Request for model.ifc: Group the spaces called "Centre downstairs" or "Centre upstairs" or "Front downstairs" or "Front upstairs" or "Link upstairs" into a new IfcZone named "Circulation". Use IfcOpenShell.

First a look at what the model holds.

```python
import ifcopenshell

model = ifcopenshell.open("model.ifc")
print(model.schema)
seen = {}
for space in model.by_type("IfcSpace"):
    seen[space.Name] = seen.get(space.Name, 0) + 1
for name, count in sorted(seen.items(), key=str):
    print(count, "x", name)
print("zones:", [z.Name for z in model.by_type("IfcZone")][:20])
```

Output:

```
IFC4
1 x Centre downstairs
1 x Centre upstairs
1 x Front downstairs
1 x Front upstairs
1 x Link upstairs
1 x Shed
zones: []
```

```python
import ifcopenshell
import ifcopenshell.api.group
import ifcopenshell.api.root

model = ifcopenshell.open("model.ifc")

names = {"Centre downstairs", "Centre upstairs", "Front downstairs", "Front upstairs", "Link upstairs"}
spaces = [s for s in model.by_type("IfcSpace") if s.Name in names]

zone = ifcopenshell.api.root.create_entity(model, ifc_class="IfcZone", name="Circulation")
ifcopenshell.api.group.assign_group(model, products=spaces, group=zone)
print(len(spaces), "spaces in", zone.Name)

model.write("model_rev.ifc")
```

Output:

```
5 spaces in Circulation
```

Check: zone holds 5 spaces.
